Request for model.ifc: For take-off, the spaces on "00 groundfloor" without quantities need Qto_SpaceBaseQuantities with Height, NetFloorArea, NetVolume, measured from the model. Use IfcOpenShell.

First a look at what the model holds.

```python
import ifcopenshell
import ifcopenshell.util.element
import ifcopenshell.util.unit

model = ifcopenshell.open("model.ifc")
print(model.schema)
for unit_type in ("LENGTHUNIT", "AREAUNIT", "VOLUMEUNIT"):
    print(unit_type, ifcopenshell.util.unit.calculate_unit_scale(model, unit_type))
storey = next(s for s in model.by_type("IfcBuildingStorey") if s.Name == "00 groundfloor")
spaces = [e for e in ifcopenshell.util.element.get_decomposition(storey) if e.is_a("IfcSpace")]
for e in sorted(spaces, key=lambda e: e.id()):
    print(e.id(), e.is_a(), e.Name, list(ifcopenshell.util.element.get_psets(e, qtos_only=True)), sep=" | ")
```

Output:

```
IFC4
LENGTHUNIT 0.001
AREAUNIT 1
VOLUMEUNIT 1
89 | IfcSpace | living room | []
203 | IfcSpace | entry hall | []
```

```python
import ifcopenshell
import ifcopenshell.api.pset
import ifcopenshell.geom
import ifcopenshell.util.element
import ifcopenshell.util.shape
import ifcopenshell.util.unit

model = ifcopenshell.open("model.ifc")
unit_scale = ifcopenshell.util.unit.calculate_unit_scale(model)
area_scale = ifcopenshell.util.unit.calculate_unit_scale(model, "AREAUNIT")
volume_scale = ifcopenshell.util.unit.calculate_unit_scale(model, "VOLUMEUNIT")
settings = ifcopenshell.geom.settings()

storey = next(s for s in model.by_type("IfcBuildingStorey") if s.Name == "00 groundfloor")
spaces = [e for e in ifcopenshell.util.element.get_decomposition(storey) if e.is_a("IfcSpace")]

for e in sorted(spaces, key=lambda e: e.id()):
    if ifcopenshell.util.element.get_psets(e, qtos_only=True, should_inherit=False):
        continue
    # Geometry comes back in metres, in the element's own axes.
    shape = ifcopenshell.geom.create_shape(settings, e)
    values = {
        "Height": ifcopenshell.util.shape.get_z(shape.geometry) / unit_scale,
        "NetFloorArea": ifcopenshell.util.shape.get_footprint_area(shape.geometry) / area_scale,
        "NetVolume": ifcopenshell.util.shape.get_volume(shape.geometry) / volume_scale,
    }
    qto = ifcopenshell.api.pset.add_qto(model, product=e, name="Qto_SpaceBaseQuantities")
    ifcopenshell.api.pset.edit_qto(model, qto=qto, properties=values)
    print(e.id(), {k: round(v, 3) for k, v in values.items()})

model.write("model_edited.ifc")
```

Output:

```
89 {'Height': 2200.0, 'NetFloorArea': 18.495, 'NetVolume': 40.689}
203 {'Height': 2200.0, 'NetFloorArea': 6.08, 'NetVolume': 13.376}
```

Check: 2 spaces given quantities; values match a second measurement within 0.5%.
